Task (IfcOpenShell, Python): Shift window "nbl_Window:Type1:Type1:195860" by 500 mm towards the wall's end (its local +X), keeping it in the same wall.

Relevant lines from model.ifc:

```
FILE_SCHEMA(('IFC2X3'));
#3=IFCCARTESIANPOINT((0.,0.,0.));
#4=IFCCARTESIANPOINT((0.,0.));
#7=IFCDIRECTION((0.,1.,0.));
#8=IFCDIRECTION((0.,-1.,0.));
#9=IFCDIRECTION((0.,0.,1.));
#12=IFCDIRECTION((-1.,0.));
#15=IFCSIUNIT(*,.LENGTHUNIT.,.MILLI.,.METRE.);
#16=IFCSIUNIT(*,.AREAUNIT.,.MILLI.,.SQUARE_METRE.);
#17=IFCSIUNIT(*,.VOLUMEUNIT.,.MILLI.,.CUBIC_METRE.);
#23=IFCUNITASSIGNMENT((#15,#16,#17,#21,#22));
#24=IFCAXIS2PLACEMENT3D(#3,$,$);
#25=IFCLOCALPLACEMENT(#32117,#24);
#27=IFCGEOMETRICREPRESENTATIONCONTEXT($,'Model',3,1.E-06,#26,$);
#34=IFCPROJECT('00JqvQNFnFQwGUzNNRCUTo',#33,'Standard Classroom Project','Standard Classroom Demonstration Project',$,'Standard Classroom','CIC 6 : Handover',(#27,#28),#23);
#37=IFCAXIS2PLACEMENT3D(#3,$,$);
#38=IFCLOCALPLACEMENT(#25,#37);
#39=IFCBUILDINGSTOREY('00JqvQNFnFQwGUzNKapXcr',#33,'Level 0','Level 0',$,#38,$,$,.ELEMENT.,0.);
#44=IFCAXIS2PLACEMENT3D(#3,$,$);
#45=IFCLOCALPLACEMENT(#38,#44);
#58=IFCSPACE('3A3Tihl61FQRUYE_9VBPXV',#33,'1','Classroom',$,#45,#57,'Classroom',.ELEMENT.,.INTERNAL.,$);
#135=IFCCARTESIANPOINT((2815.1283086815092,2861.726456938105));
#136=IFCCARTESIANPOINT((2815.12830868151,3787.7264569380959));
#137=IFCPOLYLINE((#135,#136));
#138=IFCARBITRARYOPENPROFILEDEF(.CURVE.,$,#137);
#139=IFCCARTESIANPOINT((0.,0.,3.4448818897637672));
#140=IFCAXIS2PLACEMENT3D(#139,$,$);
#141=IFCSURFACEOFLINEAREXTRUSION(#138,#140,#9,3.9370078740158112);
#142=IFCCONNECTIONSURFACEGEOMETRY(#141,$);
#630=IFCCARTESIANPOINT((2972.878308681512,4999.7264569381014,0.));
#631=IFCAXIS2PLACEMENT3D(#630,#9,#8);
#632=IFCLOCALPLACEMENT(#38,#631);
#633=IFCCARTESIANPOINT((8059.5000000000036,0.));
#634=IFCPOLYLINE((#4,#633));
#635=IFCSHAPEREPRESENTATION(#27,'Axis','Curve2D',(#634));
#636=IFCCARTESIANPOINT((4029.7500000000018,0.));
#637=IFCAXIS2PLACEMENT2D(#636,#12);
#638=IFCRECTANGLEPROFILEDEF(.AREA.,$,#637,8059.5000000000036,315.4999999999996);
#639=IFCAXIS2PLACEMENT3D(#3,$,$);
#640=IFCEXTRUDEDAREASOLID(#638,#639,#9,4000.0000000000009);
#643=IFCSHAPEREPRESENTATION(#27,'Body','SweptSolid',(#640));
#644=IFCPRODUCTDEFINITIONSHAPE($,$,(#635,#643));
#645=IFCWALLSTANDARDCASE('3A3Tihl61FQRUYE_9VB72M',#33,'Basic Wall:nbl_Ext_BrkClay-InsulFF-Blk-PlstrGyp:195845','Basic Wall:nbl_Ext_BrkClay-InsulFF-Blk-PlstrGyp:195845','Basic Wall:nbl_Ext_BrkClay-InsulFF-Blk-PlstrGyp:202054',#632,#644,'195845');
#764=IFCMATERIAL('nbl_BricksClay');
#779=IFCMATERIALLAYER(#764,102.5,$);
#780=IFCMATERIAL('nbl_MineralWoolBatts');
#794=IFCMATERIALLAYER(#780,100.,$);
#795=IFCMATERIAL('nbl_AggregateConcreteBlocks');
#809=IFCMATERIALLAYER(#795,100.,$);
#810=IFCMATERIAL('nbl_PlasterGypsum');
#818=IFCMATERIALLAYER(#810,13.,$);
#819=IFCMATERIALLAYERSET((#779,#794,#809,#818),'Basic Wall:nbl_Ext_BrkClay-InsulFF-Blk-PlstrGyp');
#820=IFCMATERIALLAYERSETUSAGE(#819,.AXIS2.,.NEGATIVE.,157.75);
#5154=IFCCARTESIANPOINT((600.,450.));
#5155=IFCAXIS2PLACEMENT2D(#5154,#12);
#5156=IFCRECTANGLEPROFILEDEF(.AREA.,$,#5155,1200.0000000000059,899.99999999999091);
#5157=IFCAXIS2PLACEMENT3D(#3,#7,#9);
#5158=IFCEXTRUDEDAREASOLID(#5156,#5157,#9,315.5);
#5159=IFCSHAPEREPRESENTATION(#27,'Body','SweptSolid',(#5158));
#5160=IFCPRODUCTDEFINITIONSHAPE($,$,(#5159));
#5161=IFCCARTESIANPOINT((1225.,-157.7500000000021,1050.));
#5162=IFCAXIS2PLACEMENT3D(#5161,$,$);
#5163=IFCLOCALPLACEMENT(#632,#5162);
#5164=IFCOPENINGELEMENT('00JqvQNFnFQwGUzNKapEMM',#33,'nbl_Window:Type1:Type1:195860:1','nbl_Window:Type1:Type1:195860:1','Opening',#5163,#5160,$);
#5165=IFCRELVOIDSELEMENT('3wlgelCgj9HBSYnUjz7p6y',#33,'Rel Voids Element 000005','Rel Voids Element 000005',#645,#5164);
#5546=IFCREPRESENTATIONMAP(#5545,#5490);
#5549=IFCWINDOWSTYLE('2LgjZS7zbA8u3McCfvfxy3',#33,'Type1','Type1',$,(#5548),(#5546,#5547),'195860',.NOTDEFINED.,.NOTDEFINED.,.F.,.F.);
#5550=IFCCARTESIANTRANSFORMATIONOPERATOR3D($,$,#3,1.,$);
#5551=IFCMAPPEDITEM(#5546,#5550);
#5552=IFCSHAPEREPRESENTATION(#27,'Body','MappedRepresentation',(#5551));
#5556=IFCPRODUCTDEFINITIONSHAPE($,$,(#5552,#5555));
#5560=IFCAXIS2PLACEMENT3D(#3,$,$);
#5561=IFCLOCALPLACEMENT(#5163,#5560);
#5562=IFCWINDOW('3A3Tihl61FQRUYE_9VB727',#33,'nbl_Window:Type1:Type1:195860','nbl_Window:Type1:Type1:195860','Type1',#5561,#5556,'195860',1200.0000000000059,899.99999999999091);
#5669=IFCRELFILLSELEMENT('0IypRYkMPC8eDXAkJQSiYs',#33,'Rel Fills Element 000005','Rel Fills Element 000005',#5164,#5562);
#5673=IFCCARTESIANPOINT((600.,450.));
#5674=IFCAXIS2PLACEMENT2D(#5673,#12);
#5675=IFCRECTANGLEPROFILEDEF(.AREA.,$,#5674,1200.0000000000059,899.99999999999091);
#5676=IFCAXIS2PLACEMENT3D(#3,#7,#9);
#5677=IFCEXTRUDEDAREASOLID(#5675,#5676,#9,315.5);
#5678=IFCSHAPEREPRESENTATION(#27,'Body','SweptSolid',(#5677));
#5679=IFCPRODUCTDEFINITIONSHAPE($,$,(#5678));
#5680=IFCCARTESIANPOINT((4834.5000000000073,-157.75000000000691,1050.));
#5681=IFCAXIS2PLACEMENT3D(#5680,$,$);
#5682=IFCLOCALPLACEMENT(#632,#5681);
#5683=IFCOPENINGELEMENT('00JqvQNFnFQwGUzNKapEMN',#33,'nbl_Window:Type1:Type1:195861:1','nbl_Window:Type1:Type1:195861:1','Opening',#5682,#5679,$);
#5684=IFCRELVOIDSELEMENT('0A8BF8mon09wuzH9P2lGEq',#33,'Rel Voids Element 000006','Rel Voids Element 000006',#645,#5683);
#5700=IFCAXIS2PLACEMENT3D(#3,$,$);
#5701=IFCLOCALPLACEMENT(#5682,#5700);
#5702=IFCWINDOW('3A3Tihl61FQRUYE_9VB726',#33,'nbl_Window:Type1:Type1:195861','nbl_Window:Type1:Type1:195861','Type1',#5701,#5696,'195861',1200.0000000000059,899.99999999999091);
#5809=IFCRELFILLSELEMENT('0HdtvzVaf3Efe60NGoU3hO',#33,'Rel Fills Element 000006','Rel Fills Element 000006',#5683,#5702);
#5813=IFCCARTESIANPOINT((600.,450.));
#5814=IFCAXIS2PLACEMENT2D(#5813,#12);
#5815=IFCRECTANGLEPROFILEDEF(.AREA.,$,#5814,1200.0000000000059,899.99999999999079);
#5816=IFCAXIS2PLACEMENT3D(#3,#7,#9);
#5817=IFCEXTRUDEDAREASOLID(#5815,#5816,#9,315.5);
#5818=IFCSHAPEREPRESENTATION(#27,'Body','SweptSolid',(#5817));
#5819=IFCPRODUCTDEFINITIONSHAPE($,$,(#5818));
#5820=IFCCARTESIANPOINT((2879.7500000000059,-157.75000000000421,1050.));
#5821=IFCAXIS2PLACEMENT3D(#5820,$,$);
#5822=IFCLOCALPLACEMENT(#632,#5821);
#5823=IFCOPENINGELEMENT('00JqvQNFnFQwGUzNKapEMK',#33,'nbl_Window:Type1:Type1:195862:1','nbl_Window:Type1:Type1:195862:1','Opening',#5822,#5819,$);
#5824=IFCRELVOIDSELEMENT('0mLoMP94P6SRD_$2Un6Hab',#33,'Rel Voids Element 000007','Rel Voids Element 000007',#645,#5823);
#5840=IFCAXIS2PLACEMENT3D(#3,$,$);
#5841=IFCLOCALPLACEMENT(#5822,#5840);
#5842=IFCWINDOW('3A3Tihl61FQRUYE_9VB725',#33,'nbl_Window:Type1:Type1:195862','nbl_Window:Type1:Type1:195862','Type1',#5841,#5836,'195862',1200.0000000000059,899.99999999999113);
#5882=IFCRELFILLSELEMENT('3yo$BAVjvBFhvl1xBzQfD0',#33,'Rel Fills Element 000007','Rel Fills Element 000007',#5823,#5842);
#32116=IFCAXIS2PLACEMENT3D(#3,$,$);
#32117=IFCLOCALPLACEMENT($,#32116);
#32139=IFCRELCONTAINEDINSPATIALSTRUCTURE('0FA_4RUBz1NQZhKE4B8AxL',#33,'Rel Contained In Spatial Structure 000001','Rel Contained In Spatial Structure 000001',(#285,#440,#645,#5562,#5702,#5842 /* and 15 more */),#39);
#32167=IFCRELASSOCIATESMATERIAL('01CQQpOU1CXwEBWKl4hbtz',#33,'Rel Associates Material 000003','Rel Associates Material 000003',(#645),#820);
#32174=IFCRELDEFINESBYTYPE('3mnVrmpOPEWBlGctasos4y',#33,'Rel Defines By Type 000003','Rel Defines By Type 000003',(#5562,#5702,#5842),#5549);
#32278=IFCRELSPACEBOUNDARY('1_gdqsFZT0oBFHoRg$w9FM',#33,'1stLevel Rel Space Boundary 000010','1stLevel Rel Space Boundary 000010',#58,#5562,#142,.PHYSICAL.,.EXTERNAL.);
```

```python
import numpy as np
import ifcopenshell
import ifcopenshell.api.geometry
import ifcopenshell.util.placement
import ifcopenshell.util.unit

model = ifcopenshell.open("model.ifc")
unit_scale = ifcopenshell.util.unit.calculate_unit_scale(model)

window = model.by_guid("3A3Tihl61FQRUYE_9VB727")
opening = window.FillsVoids[0].RelatingOpeningElement
wall = opening.VoidsElements[0].RelatingBuildingElement

wall_matrix = ifcopenshell.util.placement.get_local_placement(wall.ObjectPlacement)
shift = wall_matrix[:3, 0] * 0.5 / unit_scale
before = ifcopenshell.util.placement.get_local_placement(window.ObjectPlacement)[:3, 3].copy()

# The window is placed relative to its opening, so it follows when the opening moves.
matrix = ifcopenshell.util.placement.get_local_placement(opening.ObjectPlacement)
matrix[:3, 3] += shift
ifcopenshell.api.geometry.edit_object_placement(
    model, product=opening, matrix=matrix, is_si=False, should_transform_children=True
)

# Space boundary surfaces are stored in each space's coordinates; move them too.
for rel in window.ProvidesBoundaries:
    if not rel.ConnectionGeometry:
        continue
    surface = rel.ConnectionGeometry.SurfaceOnRelatingElement
    space_matrix = ifcopenshell.util.placement.get_local_placement(rel.RelatingSpace.ObjectPlacement)
    point = np.array(surface.Position.Location.Coordinates) + space_matrix[:3, :3].T @ shift
    surface.Position = model.createIfcAxis2Placement3D(
        model.createIfcCartesianPoint(point.tolist()), surface.Position.Axis, surface.Position.RefDirection
    )

after = ifcopenshell.util.placement.get_local_placement(window.ObjectPlacement)[:3, 3]
print("window moved by", (after - before).round(3) + 0.0)

model.write("model_updated.ifc")
```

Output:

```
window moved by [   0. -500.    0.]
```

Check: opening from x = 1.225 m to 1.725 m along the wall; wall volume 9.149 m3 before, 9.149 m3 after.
